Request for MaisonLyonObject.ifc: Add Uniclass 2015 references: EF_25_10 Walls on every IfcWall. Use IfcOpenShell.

First a look at what the model holds.

```python
import ifcopenshell

model = ifcopenshell.open("MaisonLyonObject.ifc")
print(model.schema)
print("classifications:", [c.Name for c in model.by_type("IfcClassification")])
for ifc_class in ("IfcDoor", "IfcRoof", "IfcStair", "IfcWall", "IfcWindow"):
    print(ifc_class, len(model.by_type(ifc_class)))
```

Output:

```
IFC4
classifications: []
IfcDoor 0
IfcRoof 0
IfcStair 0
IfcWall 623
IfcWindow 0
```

```python
import ifcopenshell
import ifcopenshell.api.classification

model = ifcopenshell.open("MaisonLyonObject.ifc")

system = ifcopenshell.api.classification.add_classification(model, classification="Uniclass 2015")

codes = {
    "IfcWall": ("EF_25_10", "Walls"),
}
for ifc_class, (code, name) in codes.items():
    products = model.by_type(ifc_class)
    ifcopenshell.api.classification.add_reference(
        model, products=products, classification=system, identification=code, name=name
    )
    print(code, len(products))

model.write("MaisonLyonObject_edited.ifc")
```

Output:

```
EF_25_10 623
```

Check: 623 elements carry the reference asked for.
